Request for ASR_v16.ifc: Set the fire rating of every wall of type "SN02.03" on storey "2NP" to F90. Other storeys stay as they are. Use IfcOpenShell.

First a look at what the model holds.

```python
import ifcopenshell
import ifcopenshell.util.element

model = ifcopenshell.open("ASR_v16.ifc")
print(model.schema)
storey = next(s for s in model.by_type("IfcBuildingStorey") if s.Name == "2NP")
walls = [e for e in ifcopenshell.util.element.get_decomposition(storey) if e.is_a("IfcWall")]
seen = {}
for e in walls:
    element_type = ifcopenshell.util.element.get_type(e)
    key = (element_type.Name if element_type != e and element_type else None, ifcopenshell.util.element.get_pset(e, "Pset_WallCommon", "FireRating"))
    seen[key] = seen.get(key, 0) + 1
for (name, value), count in sorted(seen.items(), key=str):
    print(count, "x", name, "|", value)
```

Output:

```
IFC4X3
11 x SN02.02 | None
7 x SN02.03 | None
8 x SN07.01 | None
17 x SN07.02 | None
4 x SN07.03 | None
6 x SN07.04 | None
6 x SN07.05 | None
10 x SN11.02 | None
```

```python
import ifcopenshell
import ifcopenshell.api.pset
import ifcopenshell.util.element

model = ifcopenshell.open("ASR_v16.ifc")

storey = next(s for s in model.by_type("IfcBuildingStorey") if s.Name == "2NP")
walls = [e for e in ifcopenshell.util.element.get_decomposition(storey) if e.is_a("IfcWall")]

count = 0
for e in walls:
    element_type = ifcopenshell.util.element.get_type(e)
    if element_type in (None, e) or element_type.Name != "SN02.03":
        continue
    # add_pset returns the element's existing set when there is one.
    pset = ifcopenshell.api.pset.add_pset(model, product=e, name="Pset_WallCommon")
    ifcopenshell.api.pset.edit_pset(model, pset=pset, properties={"FireRating": "F90"})
    count += 1

print(count, "walls updated")

model.write("ASR_v16_updated.ifc")
```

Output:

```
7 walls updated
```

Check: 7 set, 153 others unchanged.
